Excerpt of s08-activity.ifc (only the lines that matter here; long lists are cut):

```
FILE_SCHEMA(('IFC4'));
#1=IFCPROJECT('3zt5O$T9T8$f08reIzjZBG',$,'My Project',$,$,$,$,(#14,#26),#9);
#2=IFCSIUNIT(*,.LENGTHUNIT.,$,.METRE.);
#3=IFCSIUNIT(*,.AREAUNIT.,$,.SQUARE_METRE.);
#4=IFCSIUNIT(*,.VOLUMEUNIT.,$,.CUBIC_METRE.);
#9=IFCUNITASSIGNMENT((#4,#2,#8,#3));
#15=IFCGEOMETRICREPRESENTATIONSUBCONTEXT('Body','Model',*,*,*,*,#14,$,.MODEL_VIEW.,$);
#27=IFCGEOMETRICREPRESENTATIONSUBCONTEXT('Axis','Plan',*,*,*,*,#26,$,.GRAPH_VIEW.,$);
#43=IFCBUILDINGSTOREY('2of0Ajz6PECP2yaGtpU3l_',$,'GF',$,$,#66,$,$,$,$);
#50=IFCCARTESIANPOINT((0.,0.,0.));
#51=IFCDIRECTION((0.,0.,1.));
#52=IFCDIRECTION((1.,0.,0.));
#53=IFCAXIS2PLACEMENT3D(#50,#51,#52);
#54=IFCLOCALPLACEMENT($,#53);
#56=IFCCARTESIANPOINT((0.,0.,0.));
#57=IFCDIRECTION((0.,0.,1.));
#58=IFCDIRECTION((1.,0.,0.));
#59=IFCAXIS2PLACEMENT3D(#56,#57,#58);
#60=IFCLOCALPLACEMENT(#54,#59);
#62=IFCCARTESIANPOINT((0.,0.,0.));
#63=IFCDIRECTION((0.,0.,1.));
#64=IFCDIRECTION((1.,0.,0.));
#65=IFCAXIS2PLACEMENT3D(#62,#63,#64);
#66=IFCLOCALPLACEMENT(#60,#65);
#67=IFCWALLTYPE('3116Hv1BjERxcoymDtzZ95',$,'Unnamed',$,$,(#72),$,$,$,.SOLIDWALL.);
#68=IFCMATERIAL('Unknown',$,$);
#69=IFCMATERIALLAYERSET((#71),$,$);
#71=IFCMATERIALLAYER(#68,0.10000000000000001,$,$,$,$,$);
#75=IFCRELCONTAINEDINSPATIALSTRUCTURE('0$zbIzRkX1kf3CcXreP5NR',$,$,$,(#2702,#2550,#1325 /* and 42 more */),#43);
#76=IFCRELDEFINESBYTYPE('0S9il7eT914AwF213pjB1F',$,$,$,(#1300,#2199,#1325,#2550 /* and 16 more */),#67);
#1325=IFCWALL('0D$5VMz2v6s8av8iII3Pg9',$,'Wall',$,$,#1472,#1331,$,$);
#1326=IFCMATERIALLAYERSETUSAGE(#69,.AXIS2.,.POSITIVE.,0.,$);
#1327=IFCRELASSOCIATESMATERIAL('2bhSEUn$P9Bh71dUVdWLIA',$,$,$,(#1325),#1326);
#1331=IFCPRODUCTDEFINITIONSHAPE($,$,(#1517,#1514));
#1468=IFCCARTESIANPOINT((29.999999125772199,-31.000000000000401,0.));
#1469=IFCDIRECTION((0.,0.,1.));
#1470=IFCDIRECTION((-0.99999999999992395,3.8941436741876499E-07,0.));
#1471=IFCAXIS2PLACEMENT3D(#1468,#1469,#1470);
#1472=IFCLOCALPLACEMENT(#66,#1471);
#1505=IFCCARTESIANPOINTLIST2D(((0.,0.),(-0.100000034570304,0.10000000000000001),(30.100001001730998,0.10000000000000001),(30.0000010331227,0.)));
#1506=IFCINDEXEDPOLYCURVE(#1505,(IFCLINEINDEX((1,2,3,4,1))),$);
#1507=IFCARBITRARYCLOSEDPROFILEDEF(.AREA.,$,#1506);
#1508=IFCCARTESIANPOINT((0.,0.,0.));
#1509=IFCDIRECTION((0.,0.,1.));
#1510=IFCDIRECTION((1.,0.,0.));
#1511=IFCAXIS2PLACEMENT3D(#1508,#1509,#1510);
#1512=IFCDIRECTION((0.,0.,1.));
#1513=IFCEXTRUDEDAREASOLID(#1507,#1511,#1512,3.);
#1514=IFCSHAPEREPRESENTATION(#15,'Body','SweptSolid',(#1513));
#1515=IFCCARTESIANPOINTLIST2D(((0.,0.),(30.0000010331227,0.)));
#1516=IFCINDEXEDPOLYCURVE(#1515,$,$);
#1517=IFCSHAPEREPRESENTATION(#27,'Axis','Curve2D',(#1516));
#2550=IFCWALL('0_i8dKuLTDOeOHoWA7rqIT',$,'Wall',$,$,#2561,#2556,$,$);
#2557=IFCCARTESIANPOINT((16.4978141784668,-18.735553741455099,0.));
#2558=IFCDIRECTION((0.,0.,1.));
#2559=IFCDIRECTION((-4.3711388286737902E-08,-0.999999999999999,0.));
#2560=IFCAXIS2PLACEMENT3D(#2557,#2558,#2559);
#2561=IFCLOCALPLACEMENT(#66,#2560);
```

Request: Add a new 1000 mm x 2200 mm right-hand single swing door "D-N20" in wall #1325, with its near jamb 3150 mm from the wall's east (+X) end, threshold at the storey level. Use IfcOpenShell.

```python
import numpy as np
import ifcopenshell
import ifcopenshell.api.feature
import ifcopenshell.api.geometry
import ifcopenshell.api.root
import ifcopenshell.api.spatial
import ifcopenshell.geom
import ifcopenshell.util.element
import ifcopenshell.util.placement
import ifcopenshell.util.representation
import ifcopenshell.util.shape
import ifcopenshell.util.unit

model = ifcopenshell.open("s08-activity.ifc")
unit_scale = ifcopenshell.util.unit.calculate_unit_scale(model)
settings = ifcopenshell.geom.settings()


def volume(element):
    """Net volume in cubic metres, openings subtracted."""
    shape = ifcopenshell.geom.create_shape(settings, element)
    return ifcopenshell.util.shape.get_volume(shape.geometry)


wall = model.by_id(1325)
storey = ifcopenshell.util.element.get_container(wall, ifc_class="IfcBuildingStorey")
context = ifcopenshell.util.representation.get_context(model, "Model", "Body", "MODEL_VIEW")
before = volume(wall)

width, height, from_end, sill = 1, 2.2, 3.15, 0.0  # metres

# The wall runs along its own X axis, and the end named is its -X end.
wall_shape = ifcopenshell.geom.create_shape(settings, wall)
x, y, z = ifcopenshell.util.shape.get_vertices(wall_shape.geometry).T
start = x.min() + from_end
face, thickness = float(y.min()), float(y.max() - y.min())
wall_matrix = ifcopenshell.util.placement.get_local_placement(wall.ObjectPlacement)
level = ifcopenshell.util.placement.get_local_placement(storey.ObjectPlacement)[2, 3]


def in_wall(x, y):
    """Placement at x, y metres in the wall's axes, at sill height."""
    matrix = wall_matrix.copy()
    matrix[:, 3] = wall_matrix @ np.array([x / unit_scale, y / unit_scale, 0.0, 1.0])
    matrix[2, 3] = level + sill / unit_scale
    return matrix


# Opening: a box that overshoots both wall faces by 50 mm.
opening = ifcopenshell.api.root.create_entity(model, ifc_class="IfcOpeningElement", predefined_type="OPENING")
box = ifcopenshell.api.geometry.add_wall_representation(
    model, context=context, length=width, height=height, thickness=thickness + 0.1
)
ifcopenshell.api.geometry.assign_representation(model, product=opening, representation=box)
ifcopenshell.api.geometry.edit_object_placement(model, product=opening, matrix=in_wall(start, face - 0.05), is_si=False)
ifcopenshell.api.feature.add_feature(model, feature=opening, element=wall)

door = ifcopenshell.api.root.create_entity(model, ifc_class="IfcDoor", name="D-N20", predefined_type="DOOR")
door.OverallWidth, door.OverallHeight = width / unit_scale, height / unit_scale
door.OperationType = "SINGLE_SWING_RIGHT"
body = ifcopenshell.api.geometry.add_door_representation(
    model,
    context=context,
    overall_width=door.OverallWidth,
    overall_height=door.OverallHeight,
    operation_type="SINGLE_SWING_RIGHT",
    lining_properties={"LiningDepth": thickness / unit_scale, "ThresholdDepth": thickness / unit_scale},
)
ifcopenshell.api.geometry.assign_representation(model, product=door, representation=body)
ifcopenshell.api.spatial.assign_container(model, products=[door], relating_structure=storey)
ifcopenshell.api.feature.add_filling(model, opening=opening, element=door)

# The lining spans the wall, so the door starts at the wall face.
ifcopenshell.api.geometry.edit_object_placement(model, product=door, matrix=in_wall(start, face), is_si=False)

after = volume(wall)

print(f"wall volume {before:.3f} -> {after:.3f} m3")

model.write("s08-activity_v2.ifc")
```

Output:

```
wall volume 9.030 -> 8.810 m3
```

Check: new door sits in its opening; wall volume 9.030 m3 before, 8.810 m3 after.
